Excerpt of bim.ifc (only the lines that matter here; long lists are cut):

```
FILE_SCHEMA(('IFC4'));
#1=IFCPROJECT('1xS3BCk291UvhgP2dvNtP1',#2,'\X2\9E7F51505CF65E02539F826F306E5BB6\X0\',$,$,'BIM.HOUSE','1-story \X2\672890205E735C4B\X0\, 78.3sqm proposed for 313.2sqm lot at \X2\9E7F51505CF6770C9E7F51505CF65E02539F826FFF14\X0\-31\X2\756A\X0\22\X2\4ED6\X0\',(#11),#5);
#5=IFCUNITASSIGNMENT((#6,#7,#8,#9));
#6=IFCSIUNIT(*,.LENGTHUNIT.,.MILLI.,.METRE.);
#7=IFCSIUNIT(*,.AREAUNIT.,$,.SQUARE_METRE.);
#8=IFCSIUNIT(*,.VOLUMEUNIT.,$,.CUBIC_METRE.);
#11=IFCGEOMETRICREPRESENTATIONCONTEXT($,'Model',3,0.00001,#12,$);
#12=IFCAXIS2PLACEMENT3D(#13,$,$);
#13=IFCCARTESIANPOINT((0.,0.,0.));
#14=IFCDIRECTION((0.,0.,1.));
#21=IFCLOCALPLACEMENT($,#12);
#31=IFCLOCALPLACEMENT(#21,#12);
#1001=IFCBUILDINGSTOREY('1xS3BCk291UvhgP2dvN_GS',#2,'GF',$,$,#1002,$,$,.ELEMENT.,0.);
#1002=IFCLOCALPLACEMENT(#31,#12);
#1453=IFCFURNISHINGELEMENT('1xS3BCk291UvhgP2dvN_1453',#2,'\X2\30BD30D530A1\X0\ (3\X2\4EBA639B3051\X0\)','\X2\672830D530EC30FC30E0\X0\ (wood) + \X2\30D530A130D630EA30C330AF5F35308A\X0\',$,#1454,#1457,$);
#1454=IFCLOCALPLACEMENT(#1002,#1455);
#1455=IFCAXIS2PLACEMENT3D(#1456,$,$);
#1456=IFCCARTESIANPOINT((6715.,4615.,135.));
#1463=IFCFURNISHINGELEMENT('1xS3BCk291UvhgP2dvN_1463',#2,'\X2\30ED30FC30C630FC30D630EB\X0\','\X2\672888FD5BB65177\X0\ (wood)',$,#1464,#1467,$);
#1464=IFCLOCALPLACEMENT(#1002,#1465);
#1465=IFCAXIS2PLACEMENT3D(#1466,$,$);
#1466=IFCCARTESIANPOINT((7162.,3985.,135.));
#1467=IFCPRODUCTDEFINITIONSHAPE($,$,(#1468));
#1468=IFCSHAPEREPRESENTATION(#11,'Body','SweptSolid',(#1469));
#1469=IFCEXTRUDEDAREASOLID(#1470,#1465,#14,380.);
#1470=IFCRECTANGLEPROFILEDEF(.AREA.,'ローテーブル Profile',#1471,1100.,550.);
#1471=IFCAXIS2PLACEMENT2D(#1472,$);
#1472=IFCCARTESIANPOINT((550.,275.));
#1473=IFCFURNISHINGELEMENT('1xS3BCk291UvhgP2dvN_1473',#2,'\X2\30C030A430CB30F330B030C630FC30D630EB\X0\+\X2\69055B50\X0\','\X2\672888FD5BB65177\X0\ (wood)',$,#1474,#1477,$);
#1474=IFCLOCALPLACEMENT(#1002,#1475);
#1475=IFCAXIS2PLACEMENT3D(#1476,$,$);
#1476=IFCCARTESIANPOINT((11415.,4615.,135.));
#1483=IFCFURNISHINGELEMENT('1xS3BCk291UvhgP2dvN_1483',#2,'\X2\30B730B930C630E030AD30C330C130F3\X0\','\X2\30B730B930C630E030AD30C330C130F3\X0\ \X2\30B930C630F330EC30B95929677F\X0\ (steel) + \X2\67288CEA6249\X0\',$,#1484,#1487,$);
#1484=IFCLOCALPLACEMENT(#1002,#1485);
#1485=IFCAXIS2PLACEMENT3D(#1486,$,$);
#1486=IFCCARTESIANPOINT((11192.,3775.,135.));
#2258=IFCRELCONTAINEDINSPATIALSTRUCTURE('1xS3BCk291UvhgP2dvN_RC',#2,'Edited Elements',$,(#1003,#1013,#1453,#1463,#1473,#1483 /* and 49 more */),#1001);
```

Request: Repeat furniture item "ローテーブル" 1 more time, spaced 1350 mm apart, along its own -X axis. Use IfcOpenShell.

```python
import ifcopenshell
import ifcopenshell.api.geometry
import ifcopenshell.api.root
import ifcopenshell.util.element
import ifcopenshell.util.placement

model = ifcopenshell.open("bim.ifc")


def reuse_history(source, copy):
    """copy_class also copies each property set's owner history, people and application; keep the originals."""
    for rel in copy.IsDefinedBy:
        if rel.is_a("IfcRelDefinesByProperties") and (history := rel.RelatingPropertyDefinition.OwnerHistory):
            rel.RelatingPropertyDefinition.OwnerHistory = source.OwnerHistory
            ifcopenshell.util.element.remove_deep2(model, history)


source = model.by_id(1463)
base = ifcopenshell.util.placement.get_local_placement(source.ObjectPlacement)
step = -base[:3, 0] * 1350.0

for i in range(1, 2):
    copy = ifcopenshell.api.root.copy_class(model, product=source)
    copy.Representation = ifcopenshell.util.element.copy_deep(
        model, source.Representation, exclude=["IfcGeometricRepresentationContext", "IfcRepresentationMap"]
    )
    reuse_history(source, copy)
    matrix = base.copy()
    matrix[:3, 3] += i * step
    print("added at", matrix[:3, 3].round(3) + 0.0)
    ifcopenshell.api.geometry.edit_object_placement(model, product=copy, matrix=matrix, is_si=False)

model.write("bim_rev.ifc")
```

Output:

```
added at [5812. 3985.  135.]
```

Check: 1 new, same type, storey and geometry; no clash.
